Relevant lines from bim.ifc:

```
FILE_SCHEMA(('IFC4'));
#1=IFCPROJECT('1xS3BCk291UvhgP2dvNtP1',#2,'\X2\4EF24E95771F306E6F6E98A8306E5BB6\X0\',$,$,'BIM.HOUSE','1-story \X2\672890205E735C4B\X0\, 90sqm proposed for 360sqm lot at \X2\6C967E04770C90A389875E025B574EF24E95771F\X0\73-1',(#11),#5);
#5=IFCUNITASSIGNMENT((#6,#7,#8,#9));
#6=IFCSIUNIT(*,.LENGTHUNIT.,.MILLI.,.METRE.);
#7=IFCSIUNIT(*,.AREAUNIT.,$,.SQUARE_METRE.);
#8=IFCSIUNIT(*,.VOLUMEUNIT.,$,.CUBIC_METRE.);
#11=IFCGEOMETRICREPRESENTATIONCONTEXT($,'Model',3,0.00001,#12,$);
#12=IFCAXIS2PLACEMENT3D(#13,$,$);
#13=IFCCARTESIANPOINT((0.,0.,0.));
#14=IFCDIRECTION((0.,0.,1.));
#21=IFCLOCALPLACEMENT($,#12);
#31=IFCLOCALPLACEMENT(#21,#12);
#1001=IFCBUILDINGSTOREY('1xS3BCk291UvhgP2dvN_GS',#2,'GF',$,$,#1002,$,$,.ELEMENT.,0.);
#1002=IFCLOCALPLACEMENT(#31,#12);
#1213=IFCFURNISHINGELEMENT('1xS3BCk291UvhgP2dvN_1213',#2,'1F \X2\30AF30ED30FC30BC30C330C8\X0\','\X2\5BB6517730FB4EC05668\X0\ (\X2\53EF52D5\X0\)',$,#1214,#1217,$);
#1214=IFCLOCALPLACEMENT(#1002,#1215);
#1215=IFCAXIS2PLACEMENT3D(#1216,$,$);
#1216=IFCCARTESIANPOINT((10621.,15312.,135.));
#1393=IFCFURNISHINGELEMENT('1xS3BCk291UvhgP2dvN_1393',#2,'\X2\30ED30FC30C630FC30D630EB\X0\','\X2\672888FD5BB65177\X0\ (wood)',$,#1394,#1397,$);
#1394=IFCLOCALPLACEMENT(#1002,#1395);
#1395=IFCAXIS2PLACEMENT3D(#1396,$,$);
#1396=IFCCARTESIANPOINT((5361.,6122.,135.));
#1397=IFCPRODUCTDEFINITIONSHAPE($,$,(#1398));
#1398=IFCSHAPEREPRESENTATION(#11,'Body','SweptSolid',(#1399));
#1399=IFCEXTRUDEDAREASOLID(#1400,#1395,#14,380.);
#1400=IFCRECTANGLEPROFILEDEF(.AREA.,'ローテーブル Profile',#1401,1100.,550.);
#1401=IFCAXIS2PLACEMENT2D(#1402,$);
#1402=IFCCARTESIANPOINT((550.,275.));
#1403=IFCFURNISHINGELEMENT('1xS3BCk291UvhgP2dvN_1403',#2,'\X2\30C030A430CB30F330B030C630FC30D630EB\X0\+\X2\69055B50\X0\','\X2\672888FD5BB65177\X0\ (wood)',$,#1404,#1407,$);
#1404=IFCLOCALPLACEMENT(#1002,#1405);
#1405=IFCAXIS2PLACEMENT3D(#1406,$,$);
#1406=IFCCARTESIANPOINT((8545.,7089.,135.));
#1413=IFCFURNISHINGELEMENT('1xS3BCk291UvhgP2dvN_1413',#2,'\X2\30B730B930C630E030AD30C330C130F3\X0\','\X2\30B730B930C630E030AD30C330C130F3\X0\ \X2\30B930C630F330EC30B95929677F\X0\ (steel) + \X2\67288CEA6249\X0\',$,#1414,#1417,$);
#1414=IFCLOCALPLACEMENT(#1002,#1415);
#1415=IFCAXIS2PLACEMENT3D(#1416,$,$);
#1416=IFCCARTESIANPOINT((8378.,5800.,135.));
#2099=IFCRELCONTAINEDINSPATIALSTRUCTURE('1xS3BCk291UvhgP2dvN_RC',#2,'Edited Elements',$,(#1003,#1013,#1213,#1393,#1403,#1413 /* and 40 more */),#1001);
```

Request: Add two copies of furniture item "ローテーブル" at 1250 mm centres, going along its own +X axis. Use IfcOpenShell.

```python
import ifcopenshell
import ifcopenshell.api.geometry
import ifcopenshell.api.root
import ifcopenshell.util.element
import ifcopenshell.util.placement
import ifcopenshell.util.unit

model = ifcopenshell.open("bim.ifc")
unit_scale = ifcopenshell.util.unit.calculate_unit_scale(model)


def reuse_history(source, copy):
    """copy_class also copies each property set's owner history, people and application; keep the originals."""
    for rel in copy.IsDefinedBy:
        if rel.is_a("IfcRelDefinesByProperties") and (history := rel.RelatingPropertyDefinition.OwnerHistory):
            rel.RelatingPropertyDefinition.OwnerHistory = source.OwnerHistory
            ifcopenshell.util.element.remove_deep2(model, history)


source = model.by_guid("1xS3BCk291UvhgP2dvN_1393")
base = ifcopenshell.util.placement.get_local_placement(source.ObjectPlacement)
step = base[:3, 0] * 1.25 / unit_scale

for i in range(1, 3):
    copy = ifcopenshell.api.root.copy_class(model, product=source)
    copy.Representation = ifcopenshell.util.element.copy_deep(
        model, source.Representation, exclude=["IfcGeometricRepresentationContext", "IfcRepresentationMap"]
    )
    reuse_history(source, copy)
    matrix = base.copy()
    matrix[:3, 3] += i * step
    print("added at", matrix[:3, 3].round(3) + 0.0)
    ifcopenshell.api.geometry.edit_object_placement(model, product=copy, matrix=matrix, is_si=False)

model.write("bim_edited.ifc")
```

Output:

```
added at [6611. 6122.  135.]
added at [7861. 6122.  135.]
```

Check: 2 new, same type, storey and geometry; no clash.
